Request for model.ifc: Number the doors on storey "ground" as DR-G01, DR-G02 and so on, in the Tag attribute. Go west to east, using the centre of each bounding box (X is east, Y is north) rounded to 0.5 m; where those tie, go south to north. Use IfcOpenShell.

First a look at what the model holds.

```python
import ifcopenshell
import ifcopenshell.util.element
import ifcopenshell.util.placement

model = ifcopenshell.open("model.ifc")
print(model.schema)
storey = next(s for s in model.by_type("IfcBuildingStorey") if s.Name == "ground")
doors = [e for e in ifcopenshell.util.element.get_decomposition(storey) if e.is_a("IfcDoor")]
for e in sorted(doors, key=lambda e: e.id()):
    origin = ifcopenshell.util.placement.get_local_placement(e.ObjectPlacement)[:3, 3]
    print(e.id(), e.Tag, e.Name, origin.round(2) + 0.0, sep=" | ")
```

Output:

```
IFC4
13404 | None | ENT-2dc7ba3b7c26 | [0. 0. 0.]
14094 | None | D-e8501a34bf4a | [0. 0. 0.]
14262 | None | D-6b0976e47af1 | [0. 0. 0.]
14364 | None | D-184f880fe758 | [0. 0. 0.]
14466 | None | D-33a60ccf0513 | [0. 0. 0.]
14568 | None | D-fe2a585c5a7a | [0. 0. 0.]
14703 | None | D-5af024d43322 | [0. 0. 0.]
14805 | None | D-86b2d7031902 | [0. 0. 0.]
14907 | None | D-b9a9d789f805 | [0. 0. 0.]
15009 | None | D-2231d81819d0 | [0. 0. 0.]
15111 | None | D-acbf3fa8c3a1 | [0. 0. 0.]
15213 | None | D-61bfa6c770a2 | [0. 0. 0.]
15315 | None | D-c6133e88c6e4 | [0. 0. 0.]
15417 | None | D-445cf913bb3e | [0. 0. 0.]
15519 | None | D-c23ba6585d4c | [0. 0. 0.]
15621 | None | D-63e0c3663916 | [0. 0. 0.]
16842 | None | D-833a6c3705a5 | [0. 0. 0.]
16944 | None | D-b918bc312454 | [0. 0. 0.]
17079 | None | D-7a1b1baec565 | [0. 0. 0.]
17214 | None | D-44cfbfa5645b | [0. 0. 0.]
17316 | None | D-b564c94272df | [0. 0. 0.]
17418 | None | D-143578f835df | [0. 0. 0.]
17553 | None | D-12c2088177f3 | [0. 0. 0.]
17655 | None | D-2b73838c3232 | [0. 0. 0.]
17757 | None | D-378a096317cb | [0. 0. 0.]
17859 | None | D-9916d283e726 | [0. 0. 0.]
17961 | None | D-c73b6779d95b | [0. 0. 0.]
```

```python
import ifcopenshell
import ifcopenshell.geom
import ifcopenshell.util.element
import ifcopenshell.util.shape

model = ifcopenshell.open("model.ifc")
settings = ifcopenshell.geom.settings()
settings.set("use-world-coords", True)


def centre(element):
    shape = ifcopenshell.geom.create_shape(settings, element)
    return ifcopenshell.util.shape.get_bbox_centroid(shape.geometry)


storey = next(s for s in model.by_type("IfcBuildingStorey") if s.Name == "ground")
doors = [e for e in ifcopenshell.util.element.get_decomposition(storey) if e.is_a("IfcDoor")]

# Insertion points can sit at a corner or the storey origin, so sort by the geometry (in metres).
centres = {e: centre(e) for e in doors}
doors.sort(key=lambda e: (round(centres[e][0] / 0.5), centres[e][1]))

for i, e in enumerate(doors, start=1):
    number = f"DR-G{i:02d}"
    e.Tag = number
    print(e.id(), number)

model.write("model_rev.ifc")
```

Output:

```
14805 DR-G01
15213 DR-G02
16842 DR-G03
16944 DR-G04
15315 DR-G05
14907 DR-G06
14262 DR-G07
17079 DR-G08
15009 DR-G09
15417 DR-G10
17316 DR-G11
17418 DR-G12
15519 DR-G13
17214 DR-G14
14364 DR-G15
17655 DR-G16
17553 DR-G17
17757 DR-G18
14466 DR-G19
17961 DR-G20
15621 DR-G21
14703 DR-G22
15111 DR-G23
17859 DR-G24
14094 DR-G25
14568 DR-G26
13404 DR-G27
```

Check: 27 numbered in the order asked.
